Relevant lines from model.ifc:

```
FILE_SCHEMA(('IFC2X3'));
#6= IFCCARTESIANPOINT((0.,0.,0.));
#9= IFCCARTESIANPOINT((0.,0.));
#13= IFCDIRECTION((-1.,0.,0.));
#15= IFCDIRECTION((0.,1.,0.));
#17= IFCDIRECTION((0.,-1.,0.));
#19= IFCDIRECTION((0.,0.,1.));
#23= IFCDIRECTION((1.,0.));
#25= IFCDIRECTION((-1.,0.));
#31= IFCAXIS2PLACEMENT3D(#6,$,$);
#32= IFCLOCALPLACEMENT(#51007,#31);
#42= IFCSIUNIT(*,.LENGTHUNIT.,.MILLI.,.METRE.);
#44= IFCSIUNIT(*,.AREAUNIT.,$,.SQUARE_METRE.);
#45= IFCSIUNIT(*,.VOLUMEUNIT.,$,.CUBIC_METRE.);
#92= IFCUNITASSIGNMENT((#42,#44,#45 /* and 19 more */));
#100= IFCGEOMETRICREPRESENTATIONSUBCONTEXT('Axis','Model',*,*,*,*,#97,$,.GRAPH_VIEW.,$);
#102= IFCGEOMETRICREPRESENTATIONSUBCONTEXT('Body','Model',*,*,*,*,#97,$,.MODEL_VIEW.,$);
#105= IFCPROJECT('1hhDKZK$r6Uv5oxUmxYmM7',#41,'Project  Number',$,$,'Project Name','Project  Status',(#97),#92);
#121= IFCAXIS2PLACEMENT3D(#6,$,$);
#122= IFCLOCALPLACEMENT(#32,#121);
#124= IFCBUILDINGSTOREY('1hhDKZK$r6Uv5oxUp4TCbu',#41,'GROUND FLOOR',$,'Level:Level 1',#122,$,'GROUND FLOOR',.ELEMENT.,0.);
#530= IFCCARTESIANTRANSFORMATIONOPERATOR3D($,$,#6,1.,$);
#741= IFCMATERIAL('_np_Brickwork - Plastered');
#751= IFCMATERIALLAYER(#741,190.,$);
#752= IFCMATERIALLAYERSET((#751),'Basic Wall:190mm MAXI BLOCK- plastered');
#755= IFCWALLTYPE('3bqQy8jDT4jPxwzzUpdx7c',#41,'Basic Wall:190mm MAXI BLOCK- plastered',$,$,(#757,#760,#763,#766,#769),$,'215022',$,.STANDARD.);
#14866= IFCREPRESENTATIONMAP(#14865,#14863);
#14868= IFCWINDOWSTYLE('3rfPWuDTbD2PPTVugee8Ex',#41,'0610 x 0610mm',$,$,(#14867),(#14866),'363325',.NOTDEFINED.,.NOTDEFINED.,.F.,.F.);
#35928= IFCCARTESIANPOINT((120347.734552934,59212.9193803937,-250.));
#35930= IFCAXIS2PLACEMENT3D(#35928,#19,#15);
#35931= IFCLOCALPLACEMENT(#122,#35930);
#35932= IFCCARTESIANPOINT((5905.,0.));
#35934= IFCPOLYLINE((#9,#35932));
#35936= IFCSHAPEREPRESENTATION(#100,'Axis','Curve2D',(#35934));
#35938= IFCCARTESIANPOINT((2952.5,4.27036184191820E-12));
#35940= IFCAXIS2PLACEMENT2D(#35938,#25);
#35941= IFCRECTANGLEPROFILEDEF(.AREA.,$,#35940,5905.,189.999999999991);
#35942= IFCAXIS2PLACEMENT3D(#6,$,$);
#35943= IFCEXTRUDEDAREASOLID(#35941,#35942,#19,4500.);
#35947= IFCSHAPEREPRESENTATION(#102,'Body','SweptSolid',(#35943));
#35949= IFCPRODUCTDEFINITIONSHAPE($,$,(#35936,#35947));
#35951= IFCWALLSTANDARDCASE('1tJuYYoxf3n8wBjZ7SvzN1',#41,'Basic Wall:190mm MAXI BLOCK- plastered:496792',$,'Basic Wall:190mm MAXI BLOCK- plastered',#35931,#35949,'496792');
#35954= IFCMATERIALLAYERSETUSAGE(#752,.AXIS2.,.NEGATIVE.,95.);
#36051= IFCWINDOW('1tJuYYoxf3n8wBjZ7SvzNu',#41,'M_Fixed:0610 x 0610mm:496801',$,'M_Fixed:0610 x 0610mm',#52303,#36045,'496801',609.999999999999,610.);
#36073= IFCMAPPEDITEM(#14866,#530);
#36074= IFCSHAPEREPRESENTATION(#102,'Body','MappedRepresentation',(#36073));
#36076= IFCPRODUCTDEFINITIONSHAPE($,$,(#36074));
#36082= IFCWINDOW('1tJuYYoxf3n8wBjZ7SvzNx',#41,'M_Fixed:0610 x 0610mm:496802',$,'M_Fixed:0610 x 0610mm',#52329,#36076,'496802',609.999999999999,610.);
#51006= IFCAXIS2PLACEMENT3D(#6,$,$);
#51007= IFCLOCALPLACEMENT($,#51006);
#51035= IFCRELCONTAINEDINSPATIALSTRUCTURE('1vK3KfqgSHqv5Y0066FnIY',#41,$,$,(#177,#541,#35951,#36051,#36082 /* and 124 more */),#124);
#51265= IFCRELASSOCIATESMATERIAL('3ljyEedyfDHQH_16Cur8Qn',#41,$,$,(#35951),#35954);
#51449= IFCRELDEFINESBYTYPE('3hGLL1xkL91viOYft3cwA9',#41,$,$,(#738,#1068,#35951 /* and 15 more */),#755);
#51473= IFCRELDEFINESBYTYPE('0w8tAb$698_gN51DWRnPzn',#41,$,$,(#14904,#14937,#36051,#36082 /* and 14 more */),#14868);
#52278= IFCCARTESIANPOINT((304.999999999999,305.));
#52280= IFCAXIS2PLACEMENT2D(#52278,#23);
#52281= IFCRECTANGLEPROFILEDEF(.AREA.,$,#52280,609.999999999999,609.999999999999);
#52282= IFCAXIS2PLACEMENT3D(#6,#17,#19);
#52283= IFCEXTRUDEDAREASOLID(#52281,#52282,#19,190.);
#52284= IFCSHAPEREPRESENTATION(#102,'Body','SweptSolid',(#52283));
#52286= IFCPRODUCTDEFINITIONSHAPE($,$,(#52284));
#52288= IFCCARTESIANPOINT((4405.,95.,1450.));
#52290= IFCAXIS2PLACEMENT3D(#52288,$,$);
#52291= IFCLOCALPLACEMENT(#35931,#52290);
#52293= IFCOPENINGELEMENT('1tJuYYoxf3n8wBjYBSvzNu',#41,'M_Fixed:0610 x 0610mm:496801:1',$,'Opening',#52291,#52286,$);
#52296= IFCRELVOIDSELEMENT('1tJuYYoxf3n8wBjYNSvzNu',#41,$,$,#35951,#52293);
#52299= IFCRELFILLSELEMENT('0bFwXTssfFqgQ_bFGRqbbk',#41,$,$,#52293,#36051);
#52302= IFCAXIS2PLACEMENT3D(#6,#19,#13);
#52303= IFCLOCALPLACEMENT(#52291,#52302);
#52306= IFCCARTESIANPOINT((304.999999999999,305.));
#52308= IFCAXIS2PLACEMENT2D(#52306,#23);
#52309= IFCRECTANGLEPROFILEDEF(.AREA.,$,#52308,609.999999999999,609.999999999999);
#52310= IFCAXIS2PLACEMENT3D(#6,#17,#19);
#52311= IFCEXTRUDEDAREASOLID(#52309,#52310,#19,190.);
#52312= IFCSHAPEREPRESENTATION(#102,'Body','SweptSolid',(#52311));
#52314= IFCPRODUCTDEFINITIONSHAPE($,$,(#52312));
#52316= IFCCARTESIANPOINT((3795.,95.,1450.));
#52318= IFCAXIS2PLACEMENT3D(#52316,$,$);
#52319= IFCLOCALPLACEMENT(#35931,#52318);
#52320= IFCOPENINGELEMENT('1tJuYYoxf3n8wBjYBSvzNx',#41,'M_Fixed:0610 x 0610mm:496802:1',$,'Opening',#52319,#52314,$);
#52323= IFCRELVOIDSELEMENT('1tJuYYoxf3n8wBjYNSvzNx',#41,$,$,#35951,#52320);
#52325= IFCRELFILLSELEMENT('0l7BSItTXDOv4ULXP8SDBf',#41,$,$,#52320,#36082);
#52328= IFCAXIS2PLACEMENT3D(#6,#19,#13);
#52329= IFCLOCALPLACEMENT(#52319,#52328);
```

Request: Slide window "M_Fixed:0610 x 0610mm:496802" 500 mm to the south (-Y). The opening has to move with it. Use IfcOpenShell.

```python
import ifcopenshell
import ifcopenshell.api.geometry
import ifcopenshell.util.placement
import ifcopenshell.util.unit

model = ifcopenshell.open("model.ifc")
unit_scale = ifcopenshell.util.unit.calculate_unit_scale(model)

window = model.by_guid("1tJuYYoxf3n8wBjZ7SvzNx")
opening = window.FillsVoids[0].RelatingOpeningElement
wall = opening.VoidsElements[0].RelatingBuildingElement

wall_matrix = ifcopenshell.util.placement.get_local_placement(wall.ObjectPlacement)
shift = wall_matrix[:3, 0] * -0.5 / unit_scale
before = ifcopenshell.util.placement.get_local_placement(window.ObjectPlacement)[:3, 3].copy()

# The window is placed relative to its opening, so it follows when the opening moves.
matrix = ifcopenshell.util.placement.get_local_placement(opening.ObjectPlacement)
matrix[:3, 3] += shift
ifcopenshell.api.geometry.edit_object_placement(
    model, product=opening, matrix=matrix, is_si=False, should_transform_children=True
)

after = ifcopenshell.util.placement.get_local_placement(window.ObjectPlacement)[:3, 3]
print("window moved by", (after - before).round(3) + 0.0)

model.write("model_v2.ifc")
```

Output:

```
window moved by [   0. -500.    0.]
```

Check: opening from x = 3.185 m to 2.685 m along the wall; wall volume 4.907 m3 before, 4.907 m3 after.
